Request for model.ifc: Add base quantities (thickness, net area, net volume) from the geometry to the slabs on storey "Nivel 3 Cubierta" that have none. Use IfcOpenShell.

First a look at what the model holds.

```python
import ifcopenshell
import ifcopenshell.util.element
import ifcopenshell.util.unit

model = ifcopenshell.open("model.ifc")
print(model.schema)
for unit_type in ("LENGTHUNIT", "AREAUNIT", "VOLUMEUNIT"):
    print(unit_type, ifcopenshell.util.unit.calculate_unit_scale(model, unit_type))
storey = next(s for s in model.by_type("IfcBuildingStorey") if s.Name == "Nivel 3 Cubierta")
slabs = [e for e in ifcopenshell.util.element.get_decomposition(storey) if e.is_a("IfcSlab")]
for e in sorted(slabs, key=lambda e: e.id()):
    print(e.id(), e.is_a(), e.Name, list(ifcopenshell.util.element.get_psets(e, qtos_only=True)), sep=" | ")
```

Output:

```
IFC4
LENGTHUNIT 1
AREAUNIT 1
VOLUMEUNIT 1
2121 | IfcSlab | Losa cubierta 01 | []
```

```python
import ifcopenshell
import ifcopenshell.api.pset
import ifcopenshell.geom
import ifcopenshell.util.element
import ifcopenshell.util.shape
import ifcopenshell.util.unit

model = ifcopenshell.open("model.ifc")
unit_scale = ifcopenshell.util.unit.calculate_unit_scale(model)
area_scale = ifcopenshell.util.unit.calculate_unit_scale(model, "AREAUNIT")
volume_scale = ifcopenshell.util.unit.calculate_unit_scale(model, "VOLUMEUNIT")
settings = ifcopenshell.geom.settings()

storey = next(s for s in model.by_type("IfcBuildingStorey") if s.Name == "Nivel 3 Cubierta")
slabs = [e for e in ifcopenshell.util.element.get_decomposition(storey) if e.is_a("IfcSlab")]

for e in sorted(slabs, key=lambda e: e.id()):
    if ifcopenshell.util.element.get_psets(e, qtos_only=True, should_inherit=False):
        continue
    # Geometry comes back in metres, in the element's own axes.
    shape = ifcopenshell.geom.create_shape(settings, e)
    values = {
        "Width": ifcopenshell.util.shape.get_z(shape.geometry) / unit_scale,
        "NetArea": ifcopenshell.util.shape.get_footprint_area(shape.geometry) / area_scale,
        "NetVolume": ifcopenshell.util.shape.get_volume(shape.geometry) / volume_scale,
    }
    qto = ifcopenshell.api.pset.add_qto(model, product=e, name="Qto_SlabBaseQuantities")
    ifcopenshell.api.pset.edit_qto(model, qto=qto, properties=values)
    print(e.id(), {k: round(v, 3) for k, v in values.items()})

model.write("model_updated.ifc")
```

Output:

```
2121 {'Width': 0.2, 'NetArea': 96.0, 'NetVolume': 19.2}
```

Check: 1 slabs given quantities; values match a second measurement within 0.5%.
